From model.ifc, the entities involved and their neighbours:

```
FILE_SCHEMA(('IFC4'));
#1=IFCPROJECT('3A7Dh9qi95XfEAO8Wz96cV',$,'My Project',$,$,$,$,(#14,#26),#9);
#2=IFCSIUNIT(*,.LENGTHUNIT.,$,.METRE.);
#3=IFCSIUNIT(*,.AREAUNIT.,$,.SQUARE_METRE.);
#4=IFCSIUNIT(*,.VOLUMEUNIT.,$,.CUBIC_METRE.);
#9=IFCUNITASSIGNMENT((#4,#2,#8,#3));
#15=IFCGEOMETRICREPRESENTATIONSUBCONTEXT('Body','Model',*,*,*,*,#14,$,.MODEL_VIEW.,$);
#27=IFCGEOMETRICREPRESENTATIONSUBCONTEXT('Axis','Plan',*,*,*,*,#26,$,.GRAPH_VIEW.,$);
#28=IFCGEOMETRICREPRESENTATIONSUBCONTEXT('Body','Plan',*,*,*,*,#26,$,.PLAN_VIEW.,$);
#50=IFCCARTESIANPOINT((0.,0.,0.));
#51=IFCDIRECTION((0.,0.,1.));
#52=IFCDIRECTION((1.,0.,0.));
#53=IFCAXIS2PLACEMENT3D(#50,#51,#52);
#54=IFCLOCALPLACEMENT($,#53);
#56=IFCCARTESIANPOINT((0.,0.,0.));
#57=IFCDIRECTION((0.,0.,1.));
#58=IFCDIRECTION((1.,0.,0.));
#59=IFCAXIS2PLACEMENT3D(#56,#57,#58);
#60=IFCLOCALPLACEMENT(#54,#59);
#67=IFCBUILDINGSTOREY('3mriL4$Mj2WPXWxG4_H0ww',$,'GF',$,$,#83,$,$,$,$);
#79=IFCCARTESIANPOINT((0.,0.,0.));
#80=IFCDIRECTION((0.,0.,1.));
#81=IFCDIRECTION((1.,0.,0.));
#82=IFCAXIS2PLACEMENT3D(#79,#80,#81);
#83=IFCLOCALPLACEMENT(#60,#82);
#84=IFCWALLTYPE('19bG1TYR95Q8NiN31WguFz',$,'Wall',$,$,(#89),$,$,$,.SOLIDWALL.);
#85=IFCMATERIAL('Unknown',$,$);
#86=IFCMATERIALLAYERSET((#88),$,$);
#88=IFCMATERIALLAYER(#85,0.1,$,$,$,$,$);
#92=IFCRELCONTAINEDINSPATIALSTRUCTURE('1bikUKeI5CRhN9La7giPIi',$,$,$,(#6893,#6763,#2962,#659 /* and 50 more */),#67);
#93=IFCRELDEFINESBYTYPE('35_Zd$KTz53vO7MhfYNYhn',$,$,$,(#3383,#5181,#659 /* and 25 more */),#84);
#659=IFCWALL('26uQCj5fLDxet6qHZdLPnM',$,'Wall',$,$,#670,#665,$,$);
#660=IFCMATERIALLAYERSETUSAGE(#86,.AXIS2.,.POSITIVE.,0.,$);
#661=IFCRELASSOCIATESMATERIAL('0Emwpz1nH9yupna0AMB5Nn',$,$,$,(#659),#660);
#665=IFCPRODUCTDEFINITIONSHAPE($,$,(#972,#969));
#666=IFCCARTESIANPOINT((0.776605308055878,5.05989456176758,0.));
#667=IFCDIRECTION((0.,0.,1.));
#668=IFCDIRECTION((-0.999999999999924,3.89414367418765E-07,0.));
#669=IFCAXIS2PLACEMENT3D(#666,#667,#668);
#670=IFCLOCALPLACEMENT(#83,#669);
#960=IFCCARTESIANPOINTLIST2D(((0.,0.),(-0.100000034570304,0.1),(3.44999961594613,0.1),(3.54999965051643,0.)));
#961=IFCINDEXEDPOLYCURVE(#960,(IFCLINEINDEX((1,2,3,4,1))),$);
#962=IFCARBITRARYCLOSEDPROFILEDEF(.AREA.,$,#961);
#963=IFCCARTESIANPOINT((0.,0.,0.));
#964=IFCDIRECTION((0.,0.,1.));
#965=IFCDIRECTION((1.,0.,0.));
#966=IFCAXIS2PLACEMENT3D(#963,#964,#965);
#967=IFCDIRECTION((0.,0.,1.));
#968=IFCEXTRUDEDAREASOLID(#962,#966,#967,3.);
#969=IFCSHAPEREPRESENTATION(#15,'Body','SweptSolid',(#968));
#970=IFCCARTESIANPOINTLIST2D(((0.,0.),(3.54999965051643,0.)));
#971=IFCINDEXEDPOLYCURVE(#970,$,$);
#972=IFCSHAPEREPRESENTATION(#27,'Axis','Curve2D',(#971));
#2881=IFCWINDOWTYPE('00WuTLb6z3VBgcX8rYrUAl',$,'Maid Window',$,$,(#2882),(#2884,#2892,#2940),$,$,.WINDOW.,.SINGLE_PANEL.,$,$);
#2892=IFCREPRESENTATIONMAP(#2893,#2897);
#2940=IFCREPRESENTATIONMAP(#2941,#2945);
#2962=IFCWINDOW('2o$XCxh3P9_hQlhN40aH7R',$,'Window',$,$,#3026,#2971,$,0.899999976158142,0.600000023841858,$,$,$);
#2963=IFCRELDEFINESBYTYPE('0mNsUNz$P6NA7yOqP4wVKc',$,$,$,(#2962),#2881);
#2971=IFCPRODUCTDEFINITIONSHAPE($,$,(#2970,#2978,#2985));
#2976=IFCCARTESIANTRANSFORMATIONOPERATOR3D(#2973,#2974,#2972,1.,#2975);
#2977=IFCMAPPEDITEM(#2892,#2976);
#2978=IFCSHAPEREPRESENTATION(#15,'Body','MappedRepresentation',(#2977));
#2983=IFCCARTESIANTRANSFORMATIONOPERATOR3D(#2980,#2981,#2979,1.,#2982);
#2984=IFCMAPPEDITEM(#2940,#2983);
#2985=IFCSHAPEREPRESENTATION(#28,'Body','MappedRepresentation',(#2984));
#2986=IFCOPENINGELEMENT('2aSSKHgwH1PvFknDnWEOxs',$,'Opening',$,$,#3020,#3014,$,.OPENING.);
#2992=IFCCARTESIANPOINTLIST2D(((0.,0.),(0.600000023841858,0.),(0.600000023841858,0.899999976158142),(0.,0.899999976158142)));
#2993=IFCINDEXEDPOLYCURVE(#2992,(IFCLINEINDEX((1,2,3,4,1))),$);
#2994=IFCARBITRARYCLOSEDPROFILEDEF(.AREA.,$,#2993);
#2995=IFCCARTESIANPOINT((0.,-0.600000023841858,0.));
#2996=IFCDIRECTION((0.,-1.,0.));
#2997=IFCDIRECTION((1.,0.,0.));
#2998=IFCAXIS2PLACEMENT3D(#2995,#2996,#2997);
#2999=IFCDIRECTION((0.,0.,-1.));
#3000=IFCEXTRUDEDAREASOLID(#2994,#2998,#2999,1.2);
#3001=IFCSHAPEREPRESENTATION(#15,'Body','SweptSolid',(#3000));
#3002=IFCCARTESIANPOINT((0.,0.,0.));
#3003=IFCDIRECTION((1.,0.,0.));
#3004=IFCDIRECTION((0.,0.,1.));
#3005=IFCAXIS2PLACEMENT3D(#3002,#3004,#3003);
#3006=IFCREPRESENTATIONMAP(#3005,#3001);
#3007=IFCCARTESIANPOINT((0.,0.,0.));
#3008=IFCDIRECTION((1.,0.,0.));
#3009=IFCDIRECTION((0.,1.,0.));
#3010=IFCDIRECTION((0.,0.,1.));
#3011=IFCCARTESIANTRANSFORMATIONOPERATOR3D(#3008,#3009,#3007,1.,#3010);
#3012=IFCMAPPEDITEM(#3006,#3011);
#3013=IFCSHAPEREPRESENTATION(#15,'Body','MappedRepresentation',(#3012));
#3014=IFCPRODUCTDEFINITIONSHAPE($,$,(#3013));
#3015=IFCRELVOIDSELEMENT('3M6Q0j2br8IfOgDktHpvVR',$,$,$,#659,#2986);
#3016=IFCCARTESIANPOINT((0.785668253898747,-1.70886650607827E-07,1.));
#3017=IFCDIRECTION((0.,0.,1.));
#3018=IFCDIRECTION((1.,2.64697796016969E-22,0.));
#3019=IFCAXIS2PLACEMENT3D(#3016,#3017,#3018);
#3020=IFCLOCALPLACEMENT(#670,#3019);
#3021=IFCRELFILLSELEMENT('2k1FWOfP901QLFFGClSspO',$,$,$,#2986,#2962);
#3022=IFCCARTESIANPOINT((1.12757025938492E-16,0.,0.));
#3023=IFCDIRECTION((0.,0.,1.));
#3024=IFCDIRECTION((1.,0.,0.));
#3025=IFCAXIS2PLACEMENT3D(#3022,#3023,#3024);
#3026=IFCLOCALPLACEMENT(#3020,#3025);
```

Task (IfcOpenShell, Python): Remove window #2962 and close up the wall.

```python
import ifcopenshell
import ifcopenshell.api.feature
import ifcopenshell.api.root
import ifcopenshell.geom
import ifcopenshell.util.shape

model = ifcopenshell.open("model.ifc")
settings = ifcopenshell.geom.settings()


def volume(element):
    """Net volume in cubic metres, openings subtracted."""
    shape = ifcopenshell.geom.create_shape(settings, element)
    return ifcopenshell.util.shape.get_volume(shape.geometry)


window = model.by_guid("2o$XCxh3P9_hQlhN40aH7R")
opening = window.FillsVoids[0].RelatingOpeningElement
wall = opening.VoidsElements[0].RelatingBuildingElement
before = volume(wall)

ifcopenshell.api.root.remove_product(model, product=window)
ifcopenshell.api.feature.remove_feature(model, feature=opening)

after = volume(wall)

print(f"wall volume {before:.3f} -> {after:.3f} m3")

model.write("model_edited.ifc")
```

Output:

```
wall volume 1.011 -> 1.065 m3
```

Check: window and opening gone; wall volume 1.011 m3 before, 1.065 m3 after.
